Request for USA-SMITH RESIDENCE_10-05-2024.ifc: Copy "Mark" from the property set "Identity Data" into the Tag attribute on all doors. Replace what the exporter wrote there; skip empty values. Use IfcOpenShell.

First a look at what the model holds.

```python
import ifcopenshell
import ifcopenshell.util.element

model = ifcopenshell.open("USA-SMITH RESIDENCE_10-05-2024.ifc")
print(model.schema)
doors = model.by_type("IfcDoor")
print(len(doors), "doors")
for e in doors[:8]:
    source = ifcopenshell.util.element.get_pset(e, "Identity Data", "Mark")
    target = e.Tag
    print(e.id(), repr(source), repr(target), sep=" | ")
```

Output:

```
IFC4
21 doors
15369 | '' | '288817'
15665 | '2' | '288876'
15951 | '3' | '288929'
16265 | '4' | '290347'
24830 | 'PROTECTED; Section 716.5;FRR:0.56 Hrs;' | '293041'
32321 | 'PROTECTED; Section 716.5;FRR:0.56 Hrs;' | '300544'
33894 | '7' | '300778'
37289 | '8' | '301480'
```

```python
import ifcopenshell
import ifcopenshell.util.element

model = ifcopenshell.open("USA-SMITH RESIDENCE_10-05-2024.ifc")

count = 0
for e in model.by_type("IfcDoor"):
    value = ifcopenshell.util.element.get_pset(e, "Identity Data", "Mark")
    current = e.Tag
    if not value or not value.strip() or current == value:
        continue
    e.Tag = value
    count += 1

print(count, "doors updated")

model.write("USA-SMITH RESIDENCE_10-05-2024_updated.ifc")
```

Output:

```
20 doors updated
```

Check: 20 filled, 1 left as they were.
